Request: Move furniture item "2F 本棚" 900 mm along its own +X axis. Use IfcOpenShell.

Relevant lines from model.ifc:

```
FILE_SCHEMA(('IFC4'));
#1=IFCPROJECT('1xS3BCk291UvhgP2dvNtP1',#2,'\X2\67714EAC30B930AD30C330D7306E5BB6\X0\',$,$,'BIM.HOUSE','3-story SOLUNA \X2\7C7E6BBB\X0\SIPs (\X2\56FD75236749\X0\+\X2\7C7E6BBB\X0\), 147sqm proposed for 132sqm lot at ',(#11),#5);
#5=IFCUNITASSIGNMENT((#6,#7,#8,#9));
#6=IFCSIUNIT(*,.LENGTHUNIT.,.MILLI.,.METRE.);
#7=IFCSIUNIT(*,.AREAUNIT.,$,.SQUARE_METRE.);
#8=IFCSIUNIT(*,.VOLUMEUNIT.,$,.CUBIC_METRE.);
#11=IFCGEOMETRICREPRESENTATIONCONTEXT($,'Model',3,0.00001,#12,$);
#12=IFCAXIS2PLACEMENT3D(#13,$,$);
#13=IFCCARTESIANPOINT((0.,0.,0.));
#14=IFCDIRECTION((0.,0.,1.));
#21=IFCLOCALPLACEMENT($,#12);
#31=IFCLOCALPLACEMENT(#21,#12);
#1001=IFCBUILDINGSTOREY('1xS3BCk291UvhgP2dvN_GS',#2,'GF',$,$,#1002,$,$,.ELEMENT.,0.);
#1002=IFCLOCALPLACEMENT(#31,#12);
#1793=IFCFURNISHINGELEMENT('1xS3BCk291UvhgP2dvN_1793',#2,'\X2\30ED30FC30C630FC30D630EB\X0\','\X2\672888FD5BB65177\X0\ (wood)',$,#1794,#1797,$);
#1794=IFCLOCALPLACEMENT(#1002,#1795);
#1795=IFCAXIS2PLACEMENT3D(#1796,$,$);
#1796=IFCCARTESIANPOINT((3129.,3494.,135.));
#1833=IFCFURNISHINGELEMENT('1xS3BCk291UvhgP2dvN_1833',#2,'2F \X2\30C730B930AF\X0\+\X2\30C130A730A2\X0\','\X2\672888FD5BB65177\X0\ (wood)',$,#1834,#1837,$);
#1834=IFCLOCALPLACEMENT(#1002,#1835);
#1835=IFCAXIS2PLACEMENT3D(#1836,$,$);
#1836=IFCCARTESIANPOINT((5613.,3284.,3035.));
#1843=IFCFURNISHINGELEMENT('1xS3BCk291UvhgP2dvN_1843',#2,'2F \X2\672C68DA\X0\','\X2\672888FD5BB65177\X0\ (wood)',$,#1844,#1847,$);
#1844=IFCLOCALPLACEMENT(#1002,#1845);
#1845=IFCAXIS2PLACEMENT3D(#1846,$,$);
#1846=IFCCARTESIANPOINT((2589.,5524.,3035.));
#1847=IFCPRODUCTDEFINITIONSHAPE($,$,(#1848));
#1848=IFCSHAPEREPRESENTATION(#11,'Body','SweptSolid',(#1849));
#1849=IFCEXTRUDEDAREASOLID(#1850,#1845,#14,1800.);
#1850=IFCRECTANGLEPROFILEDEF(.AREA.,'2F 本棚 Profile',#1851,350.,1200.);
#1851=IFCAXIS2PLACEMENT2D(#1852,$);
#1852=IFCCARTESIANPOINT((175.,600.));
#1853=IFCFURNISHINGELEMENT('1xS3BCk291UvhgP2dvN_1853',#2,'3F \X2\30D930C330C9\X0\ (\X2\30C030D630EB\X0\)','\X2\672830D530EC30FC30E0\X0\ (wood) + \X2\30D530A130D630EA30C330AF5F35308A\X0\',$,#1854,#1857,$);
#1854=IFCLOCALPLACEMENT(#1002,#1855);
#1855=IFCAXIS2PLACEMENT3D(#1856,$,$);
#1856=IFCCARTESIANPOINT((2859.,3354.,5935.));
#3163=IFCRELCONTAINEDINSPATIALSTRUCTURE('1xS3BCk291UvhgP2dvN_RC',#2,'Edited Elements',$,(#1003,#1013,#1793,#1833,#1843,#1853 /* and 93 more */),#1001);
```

```python
import ifcopenshell
import ifcopenshell.api.geometry
import ifcopenshell.util.placement
import ifcopenshell.util.unit

model = ifcopenshell.open("model.ifc")
unit_scale = ifcopenshell.util.unit.calculate_unit_scale(model)

item = model.by_id(1843)
matrix = ifcopenshell.util.placement.get_local_placement(item.ObjectPlacement)
matrix[:3, 3] += matrix[:3, 0] * 0.9 / unit_scale
ifcopenshell.api.geometry.edit_object_placement(model, product=item, matrix=matrix, is_si=False)

print(ifcopenshell.util.placement.get_local_placement(item.ObjectPlacement).round(3) + 0.0)

model.write("model_v2.ifc")
```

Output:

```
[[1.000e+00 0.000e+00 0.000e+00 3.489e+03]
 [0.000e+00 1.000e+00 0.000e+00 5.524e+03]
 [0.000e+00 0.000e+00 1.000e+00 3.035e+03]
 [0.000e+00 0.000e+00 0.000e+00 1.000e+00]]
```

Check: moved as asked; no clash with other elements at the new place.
